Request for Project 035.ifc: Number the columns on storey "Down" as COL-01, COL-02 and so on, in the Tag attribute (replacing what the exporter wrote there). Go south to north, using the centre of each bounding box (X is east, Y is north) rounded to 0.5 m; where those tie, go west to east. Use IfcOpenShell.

First a look at what the model holds.

```python
import ifcopenshell
import ifcopenshell.util.element
import ifcopenshell.util.placement

model = ifcopenshell.open("Project 035.ifc")
print(model.schema)
storey = next(s for s in model.by_type("IfcBuildingStorey") if s.Name == "Down")
columns = [e for e in ifcopenshell.util.element.get_decomposition(storey) if e.is_a("IfcColumn")]
for e in sorted(columns, key=lambda e: e.id()):
    origin = ifcopenshell.util.placement.get_local_placement(e.ObjectPlacement)[:3, 3]
    print(e.id(), e.Tag, e.Name, origin.round(2) + 0.0, sep=" | ")
```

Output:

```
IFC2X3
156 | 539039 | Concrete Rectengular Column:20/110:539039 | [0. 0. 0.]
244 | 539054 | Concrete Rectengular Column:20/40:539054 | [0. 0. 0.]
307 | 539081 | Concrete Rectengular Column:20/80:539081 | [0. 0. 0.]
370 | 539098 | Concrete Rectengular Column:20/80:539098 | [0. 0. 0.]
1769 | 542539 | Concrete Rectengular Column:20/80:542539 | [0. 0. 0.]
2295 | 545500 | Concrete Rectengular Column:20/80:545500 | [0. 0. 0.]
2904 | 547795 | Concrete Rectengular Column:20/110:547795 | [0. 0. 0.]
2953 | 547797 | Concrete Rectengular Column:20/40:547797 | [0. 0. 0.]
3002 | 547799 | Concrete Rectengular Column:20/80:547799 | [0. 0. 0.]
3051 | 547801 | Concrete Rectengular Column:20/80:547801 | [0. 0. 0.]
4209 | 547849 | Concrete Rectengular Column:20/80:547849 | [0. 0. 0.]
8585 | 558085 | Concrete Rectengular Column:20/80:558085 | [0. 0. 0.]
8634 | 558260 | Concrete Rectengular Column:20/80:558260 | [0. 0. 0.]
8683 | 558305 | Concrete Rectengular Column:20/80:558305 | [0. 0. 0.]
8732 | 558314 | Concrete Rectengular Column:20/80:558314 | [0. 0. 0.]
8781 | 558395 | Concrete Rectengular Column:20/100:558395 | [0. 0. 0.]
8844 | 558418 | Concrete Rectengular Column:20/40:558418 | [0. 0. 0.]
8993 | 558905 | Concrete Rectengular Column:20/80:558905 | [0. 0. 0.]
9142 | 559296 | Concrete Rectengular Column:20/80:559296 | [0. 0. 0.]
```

```python
import ifcopenshell
import ifcopenshell.geom
import ifcopenshell.util.element
import ifcopenshell.util.shape

model = ifcopenshell.open("Project 035.ifc")
settings = ifcopenshell.geom.settings()
settings.set("use-world-coords", True)


def centre(element):
    shape = ifcopenshell.geom.create_shape(settings, element)
    return ifcopenshell.util.shape.get_bbox_centroid(shape.geometry)


storey = next(s for s in model.by_type("IfcBuildingStorey") if s.Name == "Down")
columns = [e for e in ifcopenshell.util.element.get_decomposition(storey) if e.is_a("IfcColumn")]

# Insertion points can sit at a corner or the storey origin, so sort by the geometry (in metres).
centres = {e: centre(e) for e in columns}
columns.sort(key=lambda e: (round(centres[e][1] / 0.5), centres[e][0]))

for i, e in enumerate(columns, start=1):
    number = f"COL-{i:02d}"
    e.Tag = number
    print(e.id(), number)

model.write("Project 035_updated.ifc")
```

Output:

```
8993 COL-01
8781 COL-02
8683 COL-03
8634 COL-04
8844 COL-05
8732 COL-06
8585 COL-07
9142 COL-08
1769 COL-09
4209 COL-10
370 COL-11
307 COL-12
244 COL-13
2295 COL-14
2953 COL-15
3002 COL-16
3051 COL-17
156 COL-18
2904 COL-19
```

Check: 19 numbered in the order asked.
